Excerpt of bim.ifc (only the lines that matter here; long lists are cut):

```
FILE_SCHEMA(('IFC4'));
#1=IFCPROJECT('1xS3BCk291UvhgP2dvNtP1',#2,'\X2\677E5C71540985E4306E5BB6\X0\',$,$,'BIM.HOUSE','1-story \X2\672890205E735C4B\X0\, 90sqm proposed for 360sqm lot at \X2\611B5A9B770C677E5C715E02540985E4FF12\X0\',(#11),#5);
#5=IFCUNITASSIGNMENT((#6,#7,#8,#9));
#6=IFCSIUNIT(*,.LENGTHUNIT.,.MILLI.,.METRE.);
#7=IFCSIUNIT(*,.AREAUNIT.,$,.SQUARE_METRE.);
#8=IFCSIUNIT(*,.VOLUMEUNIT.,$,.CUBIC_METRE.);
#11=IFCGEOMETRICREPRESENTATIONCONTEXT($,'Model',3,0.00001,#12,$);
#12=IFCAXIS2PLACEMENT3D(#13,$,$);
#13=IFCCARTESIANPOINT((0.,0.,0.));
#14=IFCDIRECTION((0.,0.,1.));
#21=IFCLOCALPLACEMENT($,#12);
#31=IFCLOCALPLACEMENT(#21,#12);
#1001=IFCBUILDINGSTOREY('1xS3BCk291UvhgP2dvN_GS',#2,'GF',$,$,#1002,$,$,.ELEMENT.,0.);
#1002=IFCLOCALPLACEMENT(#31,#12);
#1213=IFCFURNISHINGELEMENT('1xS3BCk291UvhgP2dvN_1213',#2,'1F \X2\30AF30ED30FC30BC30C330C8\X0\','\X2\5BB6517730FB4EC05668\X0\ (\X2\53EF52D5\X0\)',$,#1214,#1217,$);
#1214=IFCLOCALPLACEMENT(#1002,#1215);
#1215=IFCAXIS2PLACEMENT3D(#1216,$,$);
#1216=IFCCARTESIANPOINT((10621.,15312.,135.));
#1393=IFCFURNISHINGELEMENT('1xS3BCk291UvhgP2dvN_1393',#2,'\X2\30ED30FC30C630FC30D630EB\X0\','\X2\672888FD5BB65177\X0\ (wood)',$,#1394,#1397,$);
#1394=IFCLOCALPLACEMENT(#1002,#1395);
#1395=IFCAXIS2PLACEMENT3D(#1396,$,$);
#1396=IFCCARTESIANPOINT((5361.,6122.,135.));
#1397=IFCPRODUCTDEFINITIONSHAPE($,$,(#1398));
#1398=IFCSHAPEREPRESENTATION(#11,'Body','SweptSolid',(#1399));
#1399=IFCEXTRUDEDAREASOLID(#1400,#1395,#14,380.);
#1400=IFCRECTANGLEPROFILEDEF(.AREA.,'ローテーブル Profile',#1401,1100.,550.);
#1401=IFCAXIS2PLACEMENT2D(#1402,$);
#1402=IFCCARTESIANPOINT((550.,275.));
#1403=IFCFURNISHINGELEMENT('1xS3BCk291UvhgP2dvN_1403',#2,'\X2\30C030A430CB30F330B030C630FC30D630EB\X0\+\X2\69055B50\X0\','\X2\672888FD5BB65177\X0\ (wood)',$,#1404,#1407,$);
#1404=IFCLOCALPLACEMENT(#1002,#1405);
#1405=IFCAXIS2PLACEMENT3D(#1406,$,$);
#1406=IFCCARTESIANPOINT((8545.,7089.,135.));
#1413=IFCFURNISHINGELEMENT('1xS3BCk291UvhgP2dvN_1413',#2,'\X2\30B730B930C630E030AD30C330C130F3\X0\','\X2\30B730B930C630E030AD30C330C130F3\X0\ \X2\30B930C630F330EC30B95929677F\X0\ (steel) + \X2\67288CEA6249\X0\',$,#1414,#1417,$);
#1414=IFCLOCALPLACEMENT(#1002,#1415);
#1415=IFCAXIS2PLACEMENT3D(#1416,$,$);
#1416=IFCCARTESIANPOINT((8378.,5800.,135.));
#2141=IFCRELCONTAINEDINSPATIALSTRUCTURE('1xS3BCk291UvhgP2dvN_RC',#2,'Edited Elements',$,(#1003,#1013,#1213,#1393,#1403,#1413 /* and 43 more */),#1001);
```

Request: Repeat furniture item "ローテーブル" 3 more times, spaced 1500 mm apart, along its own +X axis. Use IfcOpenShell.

```python
import ifcopenshell
import ifcopenshell.api.geometry
import ifcopenshell.api.root
import ifcopenshell.util.element
import ifcopenshell.util.placement

model = ifcopenshell.open("bim.ifc")


def reuse_history(source, copy):
    """copy_class also copies each property set's owner history, people and application; keep the originals."""
    for rel in copy.IsDefinedBy:
        if rel.is_a("IfcRelDefinesByProperties") and (history := rel.RelatingPropertyDefinition.OwnerHistory):
            rel.RelatingPropertyDefinition.OwnerHistory = source.OwnerHistory
            ifcopenshell.util.element.remove_deep2(model, history)


source = model.by_guid("1xS3BCk291UvhgP2dvN_1393")
base = ifcopenshell.util.placement.get_local_placement(source.ObjectPlacement)
step = base[:3, 0] * 1500.0

for i in range(1, 4):
    copy = ifcopenshell.api.root.copy_class(model, product=source)
    copy.Representation = ifcopenshell.util.element.copy_deep(
        model, source.Representation, exclude=["IfcGeometricRepresentationContext", "IfcRepresentationMap"]
    )
    reuse_history(source, copy)
    matrix = base.copy()
    matrix[:3, 3] += i * step
    print("added at", matrix[:3, 3].round(3) + 0.0)
    ifcopenshell.api.geometry.edit_object_placement(model, product=copy, matrix=matrix, is_si=False)

model.write("bim_rev.ifc")
```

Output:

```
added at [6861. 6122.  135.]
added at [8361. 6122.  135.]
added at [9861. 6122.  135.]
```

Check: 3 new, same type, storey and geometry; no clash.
